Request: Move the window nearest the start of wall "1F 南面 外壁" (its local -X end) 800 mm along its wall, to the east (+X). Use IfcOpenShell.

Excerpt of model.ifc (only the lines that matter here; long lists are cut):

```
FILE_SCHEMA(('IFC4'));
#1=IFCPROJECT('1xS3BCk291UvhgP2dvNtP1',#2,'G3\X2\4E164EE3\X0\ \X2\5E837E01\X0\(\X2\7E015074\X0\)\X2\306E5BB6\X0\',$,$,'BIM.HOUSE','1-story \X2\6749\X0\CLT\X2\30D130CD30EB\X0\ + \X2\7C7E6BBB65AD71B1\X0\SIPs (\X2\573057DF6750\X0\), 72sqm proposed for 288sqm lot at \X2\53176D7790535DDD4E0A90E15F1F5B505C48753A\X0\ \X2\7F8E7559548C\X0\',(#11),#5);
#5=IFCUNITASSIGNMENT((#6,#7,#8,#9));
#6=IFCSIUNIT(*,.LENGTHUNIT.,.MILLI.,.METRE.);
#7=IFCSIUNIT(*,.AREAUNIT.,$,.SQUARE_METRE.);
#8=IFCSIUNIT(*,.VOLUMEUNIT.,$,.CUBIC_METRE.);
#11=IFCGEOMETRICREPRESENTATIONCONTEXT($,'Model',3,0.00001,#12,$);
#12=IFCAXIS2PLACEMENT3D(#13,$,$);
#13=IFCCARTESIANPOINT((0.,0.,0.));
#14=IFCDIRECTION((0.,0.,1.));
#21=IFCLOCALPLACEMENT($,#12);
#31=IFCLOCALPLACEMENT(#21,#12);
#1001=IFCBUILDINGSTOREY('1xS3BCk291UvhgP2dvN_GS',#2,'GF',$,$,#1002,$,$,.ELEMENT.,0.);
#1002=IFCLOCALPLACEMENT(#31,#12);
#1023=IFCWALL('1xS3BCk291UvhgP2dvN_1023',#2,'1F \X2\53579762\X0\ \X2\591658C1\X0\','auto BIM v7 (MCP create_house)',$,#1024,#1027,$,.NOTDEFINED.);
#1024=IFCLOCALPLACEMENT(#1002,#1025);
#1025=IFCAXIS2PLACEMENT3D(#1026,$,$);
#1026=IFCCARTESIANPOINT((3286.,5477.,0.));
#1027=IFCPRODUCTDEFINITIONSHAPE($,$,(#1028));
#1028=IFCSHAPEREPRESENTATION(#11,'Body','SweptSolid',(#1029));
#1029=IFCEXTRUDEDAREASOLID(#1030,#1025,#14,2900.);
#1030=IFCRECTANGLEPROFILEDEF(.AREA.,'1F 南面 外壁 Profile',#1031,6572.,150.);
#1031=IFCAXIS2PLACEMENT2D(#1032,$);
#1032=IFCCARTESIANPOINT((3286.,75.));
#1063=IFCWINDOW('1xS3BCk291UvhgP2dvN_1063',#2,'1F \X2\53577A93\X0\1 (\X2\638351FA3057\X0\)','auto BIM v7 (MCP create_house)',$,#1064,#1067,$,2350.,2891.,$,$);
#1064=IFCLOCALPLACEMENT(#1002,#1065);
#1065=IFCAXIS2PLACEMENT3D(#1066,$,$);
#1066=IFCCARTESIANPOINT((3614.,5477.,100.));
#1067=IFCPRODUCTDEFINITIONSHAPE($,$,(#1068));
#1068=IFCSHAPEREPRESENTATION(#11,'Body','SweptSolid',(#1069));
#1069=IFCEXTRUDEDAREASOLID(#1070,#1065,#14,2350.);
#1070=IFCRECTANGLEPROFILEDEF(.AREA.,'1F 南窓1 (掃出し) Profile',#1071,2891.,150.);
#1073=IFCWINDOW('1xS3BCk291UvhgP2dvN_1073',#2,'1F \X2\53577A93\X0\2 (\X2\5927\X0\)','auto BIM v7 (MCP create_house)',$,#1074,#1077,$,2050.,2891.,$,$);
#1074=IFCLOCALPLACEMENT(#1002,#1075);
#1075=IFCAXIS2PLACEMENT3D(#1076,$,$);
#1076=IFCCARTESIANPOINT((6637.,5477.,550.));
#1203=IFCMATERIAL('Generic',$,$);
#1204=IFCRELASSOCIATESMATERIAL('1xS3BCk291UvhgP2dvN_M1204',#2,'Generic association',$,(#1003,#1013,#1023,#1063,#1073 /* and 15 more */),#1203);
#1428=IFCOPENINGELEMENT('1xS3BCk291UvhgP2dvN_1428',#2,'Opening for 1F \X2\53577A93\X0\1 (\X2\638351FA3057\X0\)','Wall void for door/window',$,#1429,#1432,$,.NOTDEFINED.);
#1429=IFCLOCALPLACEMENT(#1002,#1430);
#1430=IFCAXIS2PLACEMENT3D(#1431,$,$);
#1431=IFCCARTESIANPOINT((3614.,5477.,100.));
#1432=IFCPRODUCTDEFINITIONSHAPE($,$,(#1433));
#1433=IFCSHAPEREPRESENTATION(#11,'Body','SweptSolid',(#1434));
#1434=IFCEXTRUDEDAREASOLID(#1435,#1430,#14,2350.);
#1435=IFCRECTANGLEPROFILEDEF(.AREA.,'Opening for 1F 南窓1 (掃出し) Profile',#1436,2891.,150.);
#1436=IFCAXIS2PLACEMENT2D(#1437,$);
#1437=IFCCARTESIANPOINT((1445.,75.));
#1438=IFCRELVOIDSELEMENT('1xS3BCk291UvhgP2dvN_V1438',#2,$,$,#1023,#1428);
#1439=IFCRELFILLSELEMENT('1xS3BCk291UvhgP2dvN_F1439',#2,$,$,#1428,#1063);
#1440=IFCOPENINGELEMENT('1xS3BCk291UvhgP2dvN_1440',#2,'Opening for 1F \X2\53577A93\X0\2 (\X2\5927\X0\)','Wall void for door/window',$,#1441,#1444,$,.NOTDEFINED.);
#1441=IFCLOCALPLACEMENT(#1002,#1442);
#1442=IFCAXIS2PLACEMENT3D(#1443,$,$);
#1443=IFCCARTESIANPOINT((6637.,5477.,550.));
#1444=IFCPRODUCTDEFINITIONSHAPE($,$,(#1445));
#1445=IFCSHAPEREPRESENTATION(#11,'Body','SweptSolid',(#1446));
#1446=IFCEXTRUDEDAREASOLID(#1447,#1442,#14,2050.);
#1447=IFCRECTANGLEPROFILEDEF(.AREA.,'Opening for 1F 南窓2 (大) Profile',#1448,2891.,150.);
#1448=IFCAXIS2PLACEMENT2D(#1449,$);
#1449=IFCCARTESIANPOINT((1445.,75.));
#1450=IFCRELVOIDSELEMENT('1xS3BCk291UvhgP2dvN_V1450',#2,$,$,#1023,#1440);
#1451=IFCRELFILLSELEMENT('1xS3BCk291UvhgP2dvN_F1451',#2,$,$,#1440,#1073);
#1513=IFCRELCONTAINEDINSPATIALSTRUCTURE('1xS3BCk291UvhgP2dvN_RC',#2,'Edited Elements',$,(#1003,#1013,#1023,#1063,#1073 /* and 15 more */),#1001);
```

```python
import ifcopenshell
import ifcopenshell.api.geometry
import ifcopenshell.util.placement
import ifcopenshell.util.unit

model = ifcopenshell.open("model.ifc")
unit_scale = ifcopenshell.util.unit.calculate_unit_scale(model)

window = model.by_guid("1xS3BCk291UvhgP2dvN_1063")
opening = window.FillsVoids[0].RelatingOpeningElement
wall = opening.VoidsElements[0].RelatingBuildingElement

wall_matrix = ifcopenshell.util.placement.get_local_placement(wall.ObjectPlacement)
shift = wall_matrix[:3, 0] * 0.8 / unit_scale
before = ifcopenshell.util.placement.get_local_placement(window.ObjectPlacement)[:3, 3].copy()

# The window is not placed relative to its opening, so move both.
for product in (opening, window):
    matrix = ifcopenshell.util.placement.get_local_placement(product.ObjectPlacement)
    matrix[:3, 3] += shift
    ifcopenshell.api.geometry.edit_object_placement(model, product=product, matrix=matrix, is_si=False)

after = ifcopenshell.util.placement.get_local_placement(window.ObjectPlacement)[:3, 3]
print("window moved by", (after - before).round(3) + 0.0)

model.write("model_edited.ifc")
```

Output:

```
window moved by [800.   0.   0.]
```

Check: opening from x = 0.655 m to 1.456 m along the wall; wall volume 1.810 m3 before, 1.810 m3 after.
